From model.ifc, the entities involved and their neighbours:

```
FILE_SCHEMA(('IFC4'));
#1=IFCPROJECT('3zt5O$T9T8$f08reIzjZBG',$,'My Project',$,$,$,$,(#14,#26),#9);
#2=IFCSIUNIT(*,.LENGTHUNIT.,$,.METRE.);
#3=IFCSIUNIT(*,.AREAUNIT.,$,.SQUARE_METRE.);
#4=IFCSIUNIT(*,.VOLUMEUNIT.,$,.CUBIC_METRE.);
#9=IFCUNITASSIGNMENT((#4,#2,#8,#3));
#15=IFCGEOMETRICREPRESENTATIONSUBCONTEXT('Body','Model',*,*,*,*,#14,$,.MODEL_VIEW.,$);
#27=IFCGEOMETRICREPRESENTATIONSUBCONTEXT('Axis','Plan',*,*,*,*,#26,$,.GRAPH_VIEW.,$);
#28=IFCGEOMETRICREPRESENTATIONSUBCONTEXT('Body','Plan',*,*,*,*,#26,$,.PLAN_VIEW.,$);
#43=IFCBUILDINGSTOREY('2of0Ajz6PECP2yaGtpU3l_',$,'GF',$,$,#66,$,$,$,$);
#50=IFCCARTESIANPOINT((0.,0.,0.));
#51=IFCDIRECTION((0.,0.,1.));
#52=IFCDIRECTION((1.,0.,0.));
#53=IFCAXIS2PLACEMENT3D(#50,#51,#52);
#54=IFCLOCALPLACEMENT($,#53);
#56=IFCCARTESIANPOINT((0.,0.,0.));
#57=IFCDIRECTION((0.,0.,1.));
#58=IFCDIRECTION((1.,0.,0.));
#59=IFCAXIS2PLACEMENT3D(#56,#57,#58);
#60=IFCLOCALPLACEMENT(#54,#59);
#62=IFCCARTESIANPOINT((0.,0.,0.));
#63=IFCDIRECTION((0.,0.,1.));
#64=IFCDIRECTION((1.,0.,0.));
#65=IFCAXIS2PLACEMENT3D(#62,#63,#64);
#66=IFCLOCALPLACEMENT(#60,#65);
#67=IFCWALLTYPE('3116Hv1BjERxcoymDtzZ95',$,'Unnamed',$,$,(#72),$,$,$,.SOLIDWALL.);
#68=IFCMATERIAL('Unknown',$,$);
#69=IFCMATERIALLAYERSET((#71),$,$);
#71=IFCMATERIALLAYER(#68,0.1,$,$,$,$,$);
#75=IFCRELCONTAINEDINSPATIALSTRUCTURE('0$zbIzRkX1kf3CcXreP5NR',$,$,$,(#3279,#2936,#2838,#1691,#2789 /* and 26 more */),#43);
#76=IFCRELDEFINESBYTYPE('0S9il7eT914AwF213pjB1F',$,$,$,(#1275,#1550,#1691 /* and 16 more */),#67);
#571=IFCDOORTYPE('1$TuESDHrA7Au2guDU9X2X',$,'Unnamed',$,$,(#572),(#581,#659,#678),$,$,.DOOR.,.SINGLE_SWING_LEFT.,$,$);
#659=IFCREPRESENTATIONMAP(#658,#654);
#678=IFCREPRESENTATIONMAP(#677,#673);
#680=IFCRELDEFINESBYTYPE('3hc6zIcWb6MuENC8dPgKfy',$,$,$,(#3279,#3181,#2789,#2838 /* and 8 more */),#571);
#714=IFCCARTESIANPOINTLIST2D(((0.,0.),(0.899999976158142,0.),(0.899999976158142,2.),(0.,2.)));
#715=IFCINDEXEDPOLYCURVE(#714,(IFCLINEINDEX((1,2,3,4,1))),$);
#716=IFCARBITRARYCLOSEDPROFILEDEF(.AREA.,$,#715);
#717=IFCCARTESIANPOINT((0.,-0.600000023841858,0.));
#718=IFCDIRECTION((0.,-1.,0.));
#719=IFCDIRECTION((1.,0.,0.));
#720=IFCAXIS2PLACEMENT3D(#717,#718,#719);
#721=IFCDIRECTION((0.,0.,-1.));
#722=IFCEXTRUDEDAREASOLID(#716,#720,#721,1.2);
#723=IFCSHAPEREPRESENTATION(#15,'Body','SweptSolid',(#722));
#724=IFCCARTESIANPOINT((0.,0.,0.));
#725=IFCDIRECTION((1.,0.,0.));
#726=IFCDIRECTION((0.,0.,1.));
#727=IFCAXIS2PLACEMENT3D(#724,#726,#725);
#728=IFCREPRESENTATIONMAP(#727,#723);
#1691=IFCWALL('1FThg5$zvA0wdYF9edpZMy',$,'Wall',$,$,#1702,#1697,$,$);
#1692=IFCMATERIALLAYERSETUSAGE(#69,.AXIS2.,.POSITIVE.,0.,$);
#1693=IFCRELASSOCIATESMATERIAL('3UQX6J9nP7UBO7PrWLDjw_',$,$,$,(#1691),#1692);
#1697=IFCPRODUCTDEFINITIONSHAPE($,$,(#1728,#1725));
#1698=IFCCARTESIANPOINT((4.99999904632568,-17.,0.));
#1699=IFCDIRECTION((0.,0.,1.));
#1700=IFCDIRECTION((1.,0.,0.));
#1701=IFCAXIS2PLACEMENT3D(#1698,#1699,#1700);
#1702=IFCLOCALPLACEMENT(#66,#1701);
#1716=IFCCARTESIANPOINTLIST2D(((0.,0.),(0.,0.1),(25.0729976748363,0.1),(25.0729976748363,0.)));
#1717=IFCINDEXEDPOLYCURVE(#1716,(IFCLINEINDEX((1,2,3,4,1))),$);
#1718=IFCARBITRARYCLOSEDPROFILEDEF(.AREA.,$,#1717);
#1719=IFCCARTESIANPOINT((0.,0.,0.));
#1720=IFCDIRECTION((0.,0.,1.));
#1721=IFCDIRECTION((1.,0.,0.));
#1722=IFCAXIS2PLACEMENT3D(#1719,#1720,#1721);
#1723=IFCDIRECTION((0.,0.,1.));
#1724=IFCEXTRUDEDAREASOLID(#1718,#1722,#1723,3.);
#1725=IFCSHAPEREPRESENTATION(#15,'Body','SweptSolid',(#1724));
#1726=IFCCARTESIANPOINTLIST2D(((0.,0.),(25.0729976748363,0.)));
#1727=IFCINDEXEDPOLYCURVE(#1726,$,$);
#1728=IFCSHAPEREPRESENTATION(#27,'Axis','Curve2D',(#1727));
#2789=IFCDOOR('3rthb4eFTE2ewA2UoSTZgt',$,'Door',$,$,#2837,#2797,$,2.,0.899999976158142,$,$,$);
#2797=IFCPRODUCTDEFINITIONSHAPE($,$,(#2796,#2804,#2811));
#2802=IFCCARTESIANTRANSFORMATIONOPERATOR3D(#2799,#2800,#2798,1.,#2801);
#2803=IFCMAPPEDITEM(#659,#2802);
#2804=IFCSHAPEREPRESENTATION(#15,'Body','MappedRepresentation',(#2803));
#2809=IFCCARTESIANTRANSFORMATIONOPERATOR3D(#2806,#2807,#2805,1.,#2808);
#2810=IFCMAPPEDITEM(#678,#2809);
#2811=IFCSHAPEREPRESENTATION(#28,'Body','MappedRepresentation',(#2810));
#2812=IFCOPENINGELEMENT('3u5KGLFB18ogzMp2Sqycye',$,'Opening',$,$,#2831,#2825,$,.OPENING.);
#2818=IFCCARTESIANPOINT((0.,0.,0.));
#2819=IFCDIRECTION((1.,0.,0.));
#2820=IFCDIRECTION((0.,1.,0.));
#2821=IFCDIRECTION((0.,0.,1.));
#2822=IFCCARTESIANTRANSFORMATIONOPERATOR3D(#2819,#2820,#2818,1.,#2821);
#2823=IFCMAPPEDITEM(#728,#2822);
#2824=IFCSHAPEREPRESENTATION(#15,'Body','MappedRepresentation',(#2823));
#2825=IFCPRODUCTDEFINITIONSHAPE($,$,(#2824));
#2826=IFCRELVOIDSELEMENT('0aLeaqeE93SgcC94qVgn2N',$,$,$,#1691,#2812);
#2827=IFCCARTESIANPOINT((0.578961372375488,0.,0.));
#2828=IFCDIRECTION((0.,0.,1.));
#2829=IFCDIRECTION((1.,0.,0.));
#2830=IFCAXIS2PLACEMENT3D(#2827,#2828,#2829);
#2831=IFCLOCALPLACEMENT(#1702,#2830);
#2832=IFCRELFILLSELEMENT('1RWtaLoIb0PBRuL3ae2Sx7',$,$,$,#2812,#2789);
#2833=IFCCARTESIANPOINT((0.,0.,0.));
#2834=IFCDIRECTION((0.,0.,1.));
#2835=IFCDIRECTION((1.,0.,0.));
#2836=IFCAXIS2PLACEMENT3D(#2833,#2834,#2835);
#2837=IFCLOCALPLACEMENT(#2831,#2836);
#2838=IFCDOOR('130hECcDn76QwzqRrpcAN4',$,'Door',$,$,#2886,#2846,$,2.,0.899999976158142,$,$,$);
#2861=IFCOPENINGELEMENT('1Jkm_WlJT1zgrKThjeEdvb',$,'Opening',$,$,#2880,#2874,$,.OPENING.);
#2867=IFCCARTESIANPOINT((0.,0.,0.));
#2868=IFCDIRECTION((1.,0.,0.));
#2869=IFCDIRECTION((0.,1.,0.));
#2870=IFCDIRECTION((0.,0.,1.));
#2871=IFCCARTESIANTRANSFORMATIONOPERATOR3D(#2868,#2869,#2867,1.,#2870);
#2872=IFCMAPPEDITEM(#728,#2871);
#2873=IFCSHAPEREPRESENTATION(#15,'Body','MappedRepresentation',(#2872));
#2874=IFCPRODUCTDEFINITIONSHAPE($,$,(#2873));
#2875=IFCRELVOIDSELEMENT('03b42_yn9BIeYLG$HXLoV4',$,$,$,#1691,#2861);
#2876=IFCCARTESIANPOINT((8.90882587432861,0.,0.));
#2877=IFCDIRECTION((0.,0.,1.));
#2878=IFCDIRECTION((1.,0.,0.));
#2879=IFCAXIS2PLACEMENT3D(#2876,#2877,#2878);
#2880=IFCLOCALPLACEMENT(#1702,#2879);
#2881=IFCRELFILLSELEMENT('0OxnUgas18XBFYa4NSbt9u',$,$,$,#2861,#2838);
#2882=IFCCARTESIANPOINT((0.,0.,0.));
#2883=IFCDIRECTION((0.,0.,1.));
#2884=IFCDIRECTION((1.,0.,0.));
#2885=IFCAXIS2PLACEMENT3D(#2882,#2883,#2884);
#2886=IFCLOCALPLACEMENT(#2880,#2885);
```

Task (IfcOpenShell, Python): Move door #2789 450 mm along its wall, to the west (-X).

```python
import ifcopenshell
import ifcopenshell.api.geometry
import ifcopenshell.util.placement
import ifcopenshell.util.unit

model = ifcopenshell.open("model.ifc")
unit_scale = ifcopenshell.util.unit.calculate_unit_scale(model)

door = model.by_guid("3rthb4eFTE2ewA2UoSTZgt")
opening = door.FillsVoids[0].RelatingOpeningElement
wall = opening.VoidsElements[0].RelatingBuildingElement

wall_matrix = ifcopenshell.util.placement.get_local_placement(wall.ObjectPlacement)
shift = wall_matrix[:3, 0] * -0.45 / unit_scale
before = ifcopenshell.util.placement.get_local_placement(door.ObjectPlacement)[:3, 3].copy()

# The door is placed relative to its opening, so it follows when the opening moves.
matrix = ifcopenshell.util.placement.get_local_placement(opening.ObjectPlacement)
matrix[:3, 3] += shift
ifcopenshell.api.geometry.edit_object_placement(
    model, product=opening, matrix=matrix, is_si=False, should_transform_children=True
)

after = ifcopenshell.util.placement.get_local_placement(door.ObjectPlacement)[:3, 3]
print("door moved by", (after - before).round(3) + 0.0)

model.write("model-out.ifc")
```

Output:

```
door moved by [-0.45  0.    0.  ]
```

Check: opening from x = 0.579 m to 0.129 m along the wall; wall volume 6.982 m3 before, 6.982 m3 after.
